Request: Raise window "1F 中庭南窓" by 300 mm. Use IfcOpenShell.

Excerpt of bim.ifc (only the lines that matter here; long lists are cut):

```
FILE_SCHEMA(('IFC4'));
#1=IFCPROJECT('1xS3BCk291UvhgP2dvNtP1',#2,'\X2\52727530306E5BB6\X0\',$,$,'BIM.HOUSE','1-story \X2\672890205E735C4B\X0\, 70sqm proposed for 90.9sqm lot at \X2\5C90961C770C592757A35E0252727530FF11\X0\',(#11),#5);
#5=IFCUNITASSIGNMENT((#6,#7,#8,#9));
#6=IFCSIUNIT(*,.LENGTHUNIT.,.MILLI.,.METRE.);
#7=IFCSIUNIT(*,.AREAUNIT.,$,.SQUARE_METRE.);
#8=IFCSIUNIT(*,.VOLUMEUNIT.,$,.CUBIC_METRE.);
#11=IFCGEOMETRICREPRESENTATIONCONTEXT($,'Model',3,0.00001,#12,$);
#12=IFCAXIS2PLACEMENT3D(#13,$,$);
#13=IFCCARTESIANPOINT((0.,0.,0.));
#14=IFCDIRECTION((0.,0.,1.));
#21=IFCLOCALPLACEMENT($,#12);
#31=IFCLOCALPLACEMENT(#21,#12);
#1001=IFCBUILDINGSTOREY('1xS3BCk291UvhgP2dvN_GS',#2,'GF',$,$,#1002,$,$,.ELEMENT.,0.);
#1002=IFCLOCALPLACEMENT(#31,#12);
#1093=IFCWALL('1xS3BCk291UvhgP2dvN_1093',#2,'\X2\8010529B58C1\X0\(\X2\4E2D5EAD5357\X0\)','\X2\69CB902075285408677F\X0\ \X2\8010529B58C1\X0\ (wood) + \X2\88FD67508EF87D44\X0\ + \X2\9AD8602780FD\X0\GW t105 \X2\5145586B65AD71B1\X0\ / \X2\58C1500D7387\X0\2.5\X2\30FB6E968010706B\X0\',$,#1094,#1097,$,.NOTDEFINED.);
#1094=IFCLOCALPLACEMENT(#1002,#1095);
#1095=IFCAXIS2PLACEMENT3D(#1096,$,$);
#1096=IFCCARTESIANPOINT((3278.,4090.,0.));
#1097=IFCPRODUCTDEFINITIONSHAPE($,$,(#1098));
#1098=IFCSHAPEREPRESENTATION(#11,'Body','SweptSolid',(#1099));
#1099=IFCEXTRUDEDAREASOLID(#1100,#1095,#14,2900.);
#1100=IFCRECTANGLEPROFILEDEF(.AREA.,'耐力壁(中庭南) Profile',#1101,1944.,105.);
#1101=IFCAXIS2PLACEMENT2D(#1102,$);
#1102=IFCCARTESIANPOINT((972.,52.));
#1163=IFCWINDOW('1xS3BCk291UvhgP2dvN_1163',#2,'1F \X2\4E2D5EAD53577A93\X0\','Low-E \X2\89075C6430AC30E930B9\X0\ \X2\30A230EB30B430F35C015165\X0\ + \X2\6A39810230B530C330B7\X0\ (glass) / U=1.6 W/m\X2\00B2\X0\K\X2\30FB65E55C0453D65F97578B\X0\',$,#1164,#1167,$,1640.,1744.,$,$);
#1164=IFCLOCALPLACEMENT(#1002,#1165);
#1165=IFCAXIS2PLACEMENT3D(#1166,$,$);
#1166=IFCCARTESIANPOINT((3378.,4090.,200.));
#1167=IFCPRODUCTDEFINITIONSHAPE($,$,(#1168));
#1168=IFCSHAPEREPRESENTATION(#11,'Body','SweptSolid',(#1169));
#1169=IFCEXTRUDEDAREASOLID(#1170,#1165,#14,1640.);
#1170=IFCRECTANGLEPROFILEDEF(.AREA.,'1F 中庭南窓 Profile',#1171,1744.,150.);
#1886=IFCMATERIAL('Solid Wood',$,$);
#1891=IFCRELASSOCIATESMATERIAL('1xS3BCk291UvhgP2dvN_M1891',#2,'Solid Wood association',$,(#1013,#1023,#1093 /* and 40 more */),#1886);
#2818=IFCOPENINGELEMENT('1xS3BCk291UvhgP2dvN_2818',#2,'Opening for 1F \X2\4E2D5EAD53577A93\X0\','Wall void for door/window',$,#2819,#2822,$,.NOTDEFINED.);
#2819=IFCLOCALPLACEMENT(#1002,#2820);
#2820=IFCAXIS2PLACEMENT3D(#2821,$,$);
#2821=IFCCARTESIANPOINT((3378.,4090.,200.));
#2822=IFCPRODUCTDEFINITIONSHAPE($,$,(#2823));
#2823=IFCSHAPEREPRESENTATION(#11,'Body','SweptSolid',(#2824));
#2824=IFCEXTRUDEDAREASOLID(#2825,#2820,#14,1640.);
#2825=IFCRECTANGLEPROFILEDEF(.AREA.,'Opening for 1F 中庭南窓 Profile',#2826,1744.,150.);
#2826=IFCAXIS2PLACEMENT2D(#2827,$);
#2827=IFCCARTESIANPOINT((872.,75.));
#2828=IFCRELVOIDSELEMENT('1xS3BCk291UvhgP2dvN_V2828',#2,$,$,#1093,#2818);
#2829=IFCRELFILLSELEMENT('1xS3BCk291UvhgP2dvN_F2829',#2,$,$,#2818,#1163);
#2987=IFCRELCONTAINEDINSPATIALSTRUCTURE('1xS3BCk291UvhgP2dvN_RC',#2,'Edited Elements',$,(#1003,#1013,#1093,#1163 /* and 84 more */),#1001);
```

```python
import numpy as np
import ifcopenshell
import ifcopenshell.api.geometry
import ifcopenshell.util.placement
import ifcopenshell.util.unit

model = ifcopenshell.open("bim.ifc")
unit_scale = ifcopenshell.util.unit.calculate_unit_scale(model)

window = model.by_guid("1xS3BCk291UvhgP2dvN_1163")
opening = window.FillsVoids[0].RelatingOpeningElement
dz = 0.3 / unit_scale

shift = np.array([0.0, 0.0, dz])
# The window is not placed relative to its opening, so move both.
for product in (opening, window):
    matrix = ifcopenshell.util.placement.get_local_placement(product.ObjectPlacement)
    matrix[:3, 3] += shift
    ifcopenshell.api.geometry.edit_object_placement(model, product=product, matrix=matrix, is_si=False)

print(f"moved by {dz * unit_scale:+.3f} m")

model.write("bim_rev.ifc")
```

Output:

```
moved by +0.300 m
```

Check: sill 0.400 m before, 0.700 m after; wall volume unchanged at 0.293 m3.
